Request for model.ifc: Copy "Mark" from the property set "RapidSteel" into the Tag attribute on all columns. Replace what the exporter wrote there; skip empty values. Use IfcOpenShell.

First a look at what the model holds.

```python
import ifcopenshell
import ifcopenshell.util.element

model = ifcopenshell.open("model.ifc")
print(model.schema)
columns = model.by_type("IfcColumn")
print(len(columns), "columns")
for e in columns[:8]:
    source = ifcopenshell.util.element.get_pset(e, "RapidSteel", "Mark")
    target = e.Tag
    print(e.id(), repr(source), repr(target), sep=" | ")
```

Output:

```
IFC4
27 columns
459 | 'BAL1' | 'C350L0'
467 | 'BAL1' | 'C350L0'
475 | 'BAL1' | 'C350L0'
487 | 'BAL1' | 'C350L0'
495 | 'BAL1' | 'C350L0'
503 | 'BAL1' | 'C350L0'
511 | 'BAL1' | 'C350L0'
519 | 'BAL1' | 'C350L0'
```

```python
import ifcopenshell
import ifcopenshell.util.element

model = ifcopenshell.open("model.ifc")

count = 0
for e in model.by_type("IfcColumn"):
    value = ifcopenshell.util.element.get_pset(e, "RapidSteel", "Mark")
    current = e.Tag
    if not value or not value.strip() or current == value:
        continue
    e.Tag = value
    count += 1

print(count, "columns updated")

model.write("model_edited.ifc")
```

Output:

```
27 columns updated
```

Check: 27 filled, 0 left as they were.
